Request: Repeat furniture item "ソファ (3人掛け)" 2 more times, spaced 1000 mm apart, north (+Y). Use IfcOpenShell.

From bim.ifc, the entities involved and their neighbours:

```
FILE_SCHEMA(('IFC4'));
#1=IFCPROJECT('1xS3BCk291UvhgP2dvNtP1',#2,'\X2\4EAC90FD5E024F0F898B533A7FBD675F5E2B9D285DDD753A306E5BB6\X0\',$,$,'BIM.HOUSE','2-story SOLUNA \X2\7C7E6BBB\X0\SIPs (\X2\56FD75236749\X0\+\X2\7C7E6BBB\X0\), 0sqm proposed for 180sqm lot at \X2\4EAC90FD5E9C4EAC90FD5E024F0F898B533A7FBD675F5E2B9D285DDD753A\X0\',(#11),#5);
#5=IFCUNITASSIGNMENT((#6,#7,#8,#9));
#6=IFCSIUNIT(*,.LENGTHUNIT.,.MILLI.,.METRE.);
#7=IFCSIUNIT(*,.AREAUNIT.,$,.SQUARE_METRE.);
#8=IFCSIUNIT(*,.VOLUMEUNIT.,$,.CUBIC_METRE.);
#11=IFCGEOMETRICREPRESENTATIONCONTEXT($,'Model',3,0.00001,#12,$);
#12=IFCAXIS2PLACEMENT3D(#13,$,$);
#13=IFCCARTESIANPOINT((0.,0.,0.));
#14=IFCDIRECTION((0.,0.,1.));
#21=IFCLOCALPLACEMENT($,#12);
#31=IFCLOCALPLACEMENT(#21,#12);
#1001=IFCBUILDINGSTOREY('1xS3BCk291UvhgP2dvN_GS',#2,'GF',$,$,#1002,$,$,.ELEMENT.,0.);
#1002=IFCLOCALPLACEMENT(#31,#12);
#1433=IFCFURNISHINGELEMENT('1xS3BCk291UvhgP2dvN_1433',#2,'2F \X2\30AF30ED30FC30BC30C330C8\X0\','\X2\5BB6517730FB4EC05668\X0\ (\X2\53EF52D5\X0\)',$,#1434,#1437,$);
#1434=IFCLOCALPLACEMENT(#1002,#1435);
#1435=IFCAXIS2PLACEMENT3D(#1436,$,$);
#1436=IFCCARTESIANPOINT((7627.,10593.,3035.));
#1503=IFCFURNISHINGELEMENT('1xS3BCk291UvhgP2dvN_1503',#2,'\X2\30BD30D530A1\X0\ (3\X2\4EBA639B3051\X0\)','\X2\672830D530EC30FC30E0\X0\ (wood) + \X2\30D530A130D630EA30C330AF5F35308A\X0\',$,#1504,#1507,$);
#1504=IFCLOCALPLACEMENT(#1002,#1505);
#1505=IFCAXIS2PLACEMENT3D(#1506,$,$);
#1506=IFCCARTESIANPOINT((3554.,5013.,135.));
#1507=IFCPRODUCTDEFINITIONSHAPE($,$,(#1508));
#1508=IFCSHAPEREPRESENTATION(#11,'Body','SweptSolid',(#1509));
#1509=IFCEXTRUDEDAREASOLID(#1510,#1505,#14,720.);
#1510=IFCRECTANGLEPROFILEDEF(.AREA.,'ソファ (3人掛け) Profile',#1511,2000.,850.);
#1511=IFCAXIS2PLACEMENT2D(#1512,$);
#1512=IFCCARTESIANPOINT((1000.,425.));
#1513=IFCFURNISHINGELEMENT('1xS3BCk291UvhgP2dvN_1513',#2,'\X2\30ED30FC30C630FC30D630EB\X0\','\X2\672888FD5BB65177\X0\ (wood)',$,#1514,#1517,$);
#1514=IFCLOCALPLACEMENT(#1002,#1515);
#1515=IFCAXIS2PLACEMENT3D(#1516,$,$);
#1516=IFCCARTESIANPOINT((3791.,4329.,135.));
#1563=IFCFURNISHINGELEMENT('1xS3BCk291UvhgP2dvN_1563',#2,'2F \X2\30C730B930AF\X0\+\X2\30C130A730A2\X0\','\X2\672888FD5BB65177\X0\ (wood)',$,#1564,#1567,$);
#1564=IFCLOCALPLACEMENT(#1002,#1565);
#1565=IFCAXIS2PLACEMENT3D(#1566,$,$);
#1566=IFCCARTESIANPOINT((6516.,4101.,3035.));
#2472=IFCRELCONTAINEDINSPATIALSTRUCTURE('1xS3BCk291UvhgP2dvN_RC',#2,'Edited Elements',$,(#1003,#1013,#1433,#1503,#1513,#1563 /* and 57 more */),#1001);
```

```python
import numpy as np
import ifcopenshell
import ifcopenshell.api.geometry
import ifcopenshell.api.root
import ifcopenshell.util.element
import ifcopenshell.util.placement
import ifcopenshell.util.unit

model = ifcopenshell.open("bim.ifc")
unit_scale = ifcopenshell.util.unit.calculate_unit_scale(model)


def reuse_history(source, copy):
    """copy_class also copies each property set's owner history, people and application; keep the originals."""
    for rel in copy.IsDefinedBy:
        if rel.is_a("IfcRelDefinesByProperties") and (history := rel.RelatingPropertyDefinition.OwnerHistory):
            rel.RelatingPropertyDefinition.OwnerHistory = source.OwnerHistory
            ifcopenshell.util.element.remove_deep2(model, history)


source = model.by_id(1503)
base = ifcopenshell.util.placement.get_local_placement(source.ObjectPlacement)
step = np.array([0.0, 1.0, 0.0]) * 1 / unit_scale

for i in range(1, 3):
    copy = ifcopenshell.api.root.copy_class(model, product=source)
    copy.Representation = ifcopenshell.util.element.copy_deep(
        model, source.Representation, exclude=["IfcGeometricRepresentationContext", "IfcRepresentationMap"]
    )
    reuse_history(source, copy)
    matrix = base.copy()
    matrix[:3, 3] += i * step
    print("added at", matrix[:3, 3].round(3) + 0.0)
    ifcopenshell.api.geometry.edit_object_placement(model, product=copy, matrix=matrix, is_si=False)

model.write("bim_rev.ifc")
```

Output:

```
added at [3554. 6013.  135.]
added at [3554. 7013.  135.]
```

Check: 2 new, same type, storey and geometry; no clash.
